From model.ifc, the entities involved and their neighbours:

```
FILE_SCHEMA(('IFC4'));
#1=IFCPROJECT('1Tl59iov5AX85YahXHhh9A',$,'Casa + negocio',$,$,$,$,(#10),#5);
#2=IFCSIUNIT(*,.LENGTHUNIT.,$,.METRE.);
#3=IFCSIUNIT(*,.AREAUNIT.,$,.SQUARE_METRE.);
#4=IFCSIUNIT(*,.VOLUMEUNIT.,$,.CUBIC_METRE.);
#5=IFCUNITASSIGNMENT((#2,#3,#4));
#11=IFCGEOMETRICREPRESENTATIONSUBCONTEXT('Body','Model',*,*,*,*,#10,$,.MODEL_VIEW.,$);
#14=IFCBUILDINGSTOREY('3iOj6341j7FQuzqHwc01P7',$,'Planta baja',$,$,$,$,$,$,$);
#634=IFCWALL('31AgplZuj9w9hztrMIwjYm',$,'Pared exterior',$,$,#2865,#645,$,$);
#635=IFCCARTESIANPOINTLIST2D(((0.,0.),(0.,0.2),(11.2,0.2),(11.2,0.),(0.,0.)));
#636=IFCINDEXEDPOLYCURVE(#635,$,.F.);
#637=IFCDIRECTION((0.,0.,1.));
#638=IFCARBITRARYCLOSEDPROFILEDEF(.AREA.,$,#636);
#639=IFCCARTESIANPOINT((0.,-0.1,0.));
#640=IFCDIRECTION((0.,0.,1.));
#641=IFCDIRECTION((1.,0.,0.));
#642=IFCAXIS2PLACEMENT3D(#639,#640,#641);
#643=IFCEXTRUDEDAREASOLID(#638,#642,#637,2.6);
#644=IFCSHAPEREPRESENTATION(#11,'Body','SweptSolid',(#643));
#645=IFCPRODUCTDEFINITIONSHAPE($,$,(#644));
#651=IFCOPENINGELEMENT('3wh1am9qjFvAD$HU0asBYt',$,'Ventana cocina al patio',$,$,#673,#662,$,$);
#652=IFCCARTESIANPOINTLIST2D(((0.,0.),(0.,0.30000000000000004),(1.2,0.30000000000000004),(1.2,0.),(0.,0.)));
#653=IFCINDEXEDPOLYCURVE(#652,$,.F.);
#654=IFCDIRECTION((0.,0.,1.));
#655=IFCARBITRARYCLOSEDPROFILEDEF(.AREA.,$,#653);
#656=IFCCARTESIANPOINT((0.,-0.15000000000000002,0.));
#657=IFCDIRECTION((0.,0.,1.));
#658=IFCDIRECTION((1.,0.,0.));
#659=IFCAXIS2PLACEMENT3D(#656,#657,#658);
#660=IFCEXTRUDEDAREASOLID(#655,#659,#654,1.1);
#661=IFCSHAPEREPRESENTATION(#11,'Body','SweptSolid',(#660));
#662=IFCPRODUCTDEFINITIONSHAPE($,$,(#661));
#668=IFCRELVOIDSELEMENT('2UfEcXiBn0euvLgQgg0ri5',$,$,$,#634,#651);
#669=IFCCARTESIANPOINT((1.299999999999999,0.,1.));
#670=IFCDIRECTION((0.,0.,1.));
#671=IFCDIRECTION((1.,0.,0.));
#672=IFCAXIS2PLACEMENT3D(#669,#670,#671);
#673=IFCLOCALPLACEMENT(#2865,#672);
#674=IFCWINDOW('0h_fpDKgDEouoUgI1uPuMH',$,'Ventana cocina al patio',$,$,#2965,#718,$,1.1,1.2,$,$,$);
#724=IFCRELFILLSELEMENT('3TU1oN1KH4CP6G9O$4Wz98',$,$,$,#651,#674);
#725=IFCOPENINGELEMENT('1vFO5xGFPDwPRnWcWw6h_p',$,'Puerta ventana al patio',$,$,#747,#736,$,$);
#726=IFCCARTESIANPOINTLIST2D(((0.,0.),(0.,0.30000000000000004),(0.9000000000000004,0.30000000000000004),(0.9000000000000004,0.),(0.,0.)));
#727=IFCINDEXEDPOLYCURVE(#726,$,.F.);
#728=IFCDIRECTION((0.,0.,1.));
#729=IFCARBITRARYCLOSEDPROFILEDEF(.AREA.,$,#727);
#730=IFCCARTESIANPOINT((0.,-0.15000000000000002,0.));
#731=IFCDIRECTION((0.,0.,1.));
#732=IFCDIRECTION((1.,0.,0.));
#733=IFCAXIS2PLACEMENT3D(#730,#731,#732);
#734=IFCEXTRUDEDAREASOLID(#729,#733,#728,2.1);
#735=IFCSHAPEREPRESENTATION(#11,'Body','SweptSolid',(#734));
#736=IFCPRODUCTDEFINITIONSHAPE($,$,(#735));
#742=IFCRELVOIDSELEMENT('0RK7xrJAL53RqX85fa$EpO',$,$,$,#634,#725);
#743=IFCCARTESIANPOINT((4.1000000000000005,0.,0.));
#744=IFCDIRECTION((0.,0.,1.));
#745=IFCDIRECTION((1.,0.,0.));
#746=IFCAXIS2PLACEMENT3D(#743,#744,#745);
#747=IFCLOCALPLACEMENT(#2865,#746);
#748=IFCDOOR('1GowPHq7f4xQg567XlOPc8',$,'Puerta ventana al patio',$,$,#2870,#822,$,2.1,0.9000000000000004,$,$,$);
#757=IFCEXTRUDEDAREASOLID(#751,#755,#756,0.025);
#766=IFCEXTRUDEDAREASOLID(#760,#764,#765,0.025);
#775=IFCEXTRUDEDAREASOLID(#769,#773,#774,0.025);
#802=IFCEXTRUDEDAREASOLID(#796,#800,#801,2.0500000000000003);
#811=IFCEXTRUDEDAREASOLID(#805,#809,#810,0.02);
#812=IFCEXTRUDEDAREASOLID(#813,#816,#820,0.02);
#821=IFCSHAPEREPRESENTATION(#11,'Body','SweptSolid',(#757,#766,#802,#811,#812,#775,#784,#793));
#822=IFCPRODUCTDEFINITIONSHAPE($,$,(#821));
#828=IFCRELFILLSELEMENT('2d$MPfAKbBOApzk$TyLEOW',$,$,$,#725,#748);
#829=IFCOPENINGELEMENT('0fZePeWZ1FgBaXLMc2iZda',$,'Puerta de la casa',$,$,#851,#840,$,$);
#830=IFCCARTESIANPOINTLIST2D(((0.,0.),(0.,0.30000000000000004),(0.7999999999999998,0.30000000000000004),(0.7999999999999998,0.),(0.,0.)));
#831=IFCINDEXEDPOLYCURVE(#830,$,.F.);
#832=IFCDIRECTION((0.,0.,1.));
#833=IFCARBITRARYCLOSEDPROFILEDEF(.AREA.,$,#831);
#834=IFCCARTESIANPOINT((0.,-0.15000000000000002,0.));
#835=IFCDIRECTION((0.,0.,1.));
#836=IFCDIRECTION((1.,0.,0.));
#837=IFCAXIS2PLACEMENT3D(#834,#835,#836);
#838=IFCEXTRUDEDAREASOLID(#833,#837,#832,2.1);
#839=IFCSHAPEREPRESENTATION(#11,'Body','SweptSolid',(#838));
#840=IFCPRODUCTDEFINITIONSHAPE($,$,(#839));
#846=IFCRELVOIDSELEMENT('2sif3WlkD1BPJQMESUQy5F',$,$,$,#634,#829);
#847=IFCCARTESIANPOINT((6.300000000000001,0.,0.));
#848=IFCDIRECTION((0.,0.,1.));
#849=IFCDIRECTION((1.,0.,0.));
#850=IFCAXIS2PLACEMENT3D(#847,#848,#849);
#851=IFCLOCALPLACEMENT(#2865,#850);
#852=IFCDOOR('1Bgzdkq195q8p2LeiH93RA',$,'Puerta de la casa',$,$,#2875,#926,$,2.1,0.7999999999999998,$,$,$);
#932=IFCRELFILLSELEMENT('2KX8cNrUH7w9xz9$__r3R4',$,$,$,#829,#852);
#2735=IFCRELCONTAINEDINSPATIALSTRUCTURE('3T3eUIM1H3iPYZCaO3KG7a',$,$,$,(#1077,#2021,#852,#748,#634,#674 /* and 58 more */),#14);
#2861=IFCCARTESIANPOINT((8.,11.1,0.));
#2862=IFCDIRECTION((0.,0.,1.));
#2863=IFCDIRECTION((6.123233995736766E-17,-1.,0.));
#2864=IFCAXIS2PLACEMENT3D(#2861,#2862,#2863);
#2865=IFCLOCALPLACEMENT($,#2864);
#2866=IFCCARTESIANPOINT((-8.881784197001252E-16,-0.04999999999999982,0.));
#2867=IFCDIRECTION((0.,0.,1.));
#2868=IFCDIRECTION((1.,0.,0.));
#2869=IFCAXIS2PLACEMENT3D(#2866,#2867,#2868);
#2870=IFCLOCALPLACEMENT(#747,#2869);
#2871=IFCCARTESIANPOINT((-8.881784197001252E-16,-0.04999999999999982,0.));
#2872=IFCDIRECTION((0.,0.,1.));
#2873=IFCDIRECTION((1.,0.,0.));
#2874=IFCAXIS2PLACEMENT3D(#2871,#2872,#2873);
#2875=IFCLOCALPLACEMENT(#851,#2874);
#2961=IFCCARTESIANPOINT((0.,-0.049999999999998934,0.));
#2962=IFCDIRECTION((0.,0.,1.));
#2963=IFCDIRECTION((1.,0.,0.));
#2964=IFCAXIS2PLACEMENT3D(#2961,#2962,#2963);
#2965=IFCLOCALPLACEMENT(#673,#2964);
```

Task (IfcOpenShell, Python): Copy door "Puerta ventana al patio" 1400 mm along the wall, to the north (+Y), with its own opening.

```python
import ifcopenshell
import ifcopenshell.api.feature
import ifcopenshell.api.geometry
import ifcopenshell.api.root
import ifcopenshell.geom
import ifcopenshell.util.element
import ifcopenshell.util.placement
import ifcopenshell.util.shape
import ifcopenshell.util.unit

model = ifcopenshell.open("model.ifc")
unit_scale = ifcopenshell.util.unit.calculate_unit_scale(model)
settings = ifcopenshell.geom.settings()


def volume(element):
    """Net volume in cubic metres, openings subtracted."""
    shape = ifcopenshell.geom.create_shape(settings, element)
    return ifcopenshell.util.shape.get_volume(shape.geometry)


door = model.by_guid("1GowPHq7f4xQg567XlOPc8")
opening = door.FillsVoids[0].RelatingOpeningElement
wall = opening.VoidsElements[0].RelatingBuildingElement
before = volume(wall)
shift = ifcopenshell.util.placement.get_local_placement(wall.ObjectPlacement)[:3, 0] * -1.4 / unit_scale

# copy_class copies the void relationship, type, container and properties, but no geometry.
new_opening = ifcopenshell.api.root.copy_class(model, product=opening)
new_opening.Representation = ifcopenshell.util.element.copy_deep(
    model, opening.Representation, exclude=["IfcGeometricRepresentationContext", "IfcRepresentationMap"]
)
new_door = ifcopenshell.api.root.copy_class(model, product=door)
new_door.Representation = ifcopenshell.util.element.copy_deep(
    model, door.Representation, exclude=["IfcGeometricRepresentationContext", "IfcRepresentationMap"]
)
ifcopenshell.api.feature.add_filling(model, opening=new_opening, element=new_door)

for old, new in ((opening, new_opening), (door, new_door)):
    matrix = ifcopenshell.util.placement.get_local_placement(old.ObjectPlacement)
    matrix[:3, 3] += shift
    ifcopenshell.api.geometry.edit_object_placement(model, product=new, matrix=matrix, is_si=False)

after = volume(wall)

print(f"wall volume {before:.3f} -> {after:.3f} m3")

model.write("model_updated.ifc")
```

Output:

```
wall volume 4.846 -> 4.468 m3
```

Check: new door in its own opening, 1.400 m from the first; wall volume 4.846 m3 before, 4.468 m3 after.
